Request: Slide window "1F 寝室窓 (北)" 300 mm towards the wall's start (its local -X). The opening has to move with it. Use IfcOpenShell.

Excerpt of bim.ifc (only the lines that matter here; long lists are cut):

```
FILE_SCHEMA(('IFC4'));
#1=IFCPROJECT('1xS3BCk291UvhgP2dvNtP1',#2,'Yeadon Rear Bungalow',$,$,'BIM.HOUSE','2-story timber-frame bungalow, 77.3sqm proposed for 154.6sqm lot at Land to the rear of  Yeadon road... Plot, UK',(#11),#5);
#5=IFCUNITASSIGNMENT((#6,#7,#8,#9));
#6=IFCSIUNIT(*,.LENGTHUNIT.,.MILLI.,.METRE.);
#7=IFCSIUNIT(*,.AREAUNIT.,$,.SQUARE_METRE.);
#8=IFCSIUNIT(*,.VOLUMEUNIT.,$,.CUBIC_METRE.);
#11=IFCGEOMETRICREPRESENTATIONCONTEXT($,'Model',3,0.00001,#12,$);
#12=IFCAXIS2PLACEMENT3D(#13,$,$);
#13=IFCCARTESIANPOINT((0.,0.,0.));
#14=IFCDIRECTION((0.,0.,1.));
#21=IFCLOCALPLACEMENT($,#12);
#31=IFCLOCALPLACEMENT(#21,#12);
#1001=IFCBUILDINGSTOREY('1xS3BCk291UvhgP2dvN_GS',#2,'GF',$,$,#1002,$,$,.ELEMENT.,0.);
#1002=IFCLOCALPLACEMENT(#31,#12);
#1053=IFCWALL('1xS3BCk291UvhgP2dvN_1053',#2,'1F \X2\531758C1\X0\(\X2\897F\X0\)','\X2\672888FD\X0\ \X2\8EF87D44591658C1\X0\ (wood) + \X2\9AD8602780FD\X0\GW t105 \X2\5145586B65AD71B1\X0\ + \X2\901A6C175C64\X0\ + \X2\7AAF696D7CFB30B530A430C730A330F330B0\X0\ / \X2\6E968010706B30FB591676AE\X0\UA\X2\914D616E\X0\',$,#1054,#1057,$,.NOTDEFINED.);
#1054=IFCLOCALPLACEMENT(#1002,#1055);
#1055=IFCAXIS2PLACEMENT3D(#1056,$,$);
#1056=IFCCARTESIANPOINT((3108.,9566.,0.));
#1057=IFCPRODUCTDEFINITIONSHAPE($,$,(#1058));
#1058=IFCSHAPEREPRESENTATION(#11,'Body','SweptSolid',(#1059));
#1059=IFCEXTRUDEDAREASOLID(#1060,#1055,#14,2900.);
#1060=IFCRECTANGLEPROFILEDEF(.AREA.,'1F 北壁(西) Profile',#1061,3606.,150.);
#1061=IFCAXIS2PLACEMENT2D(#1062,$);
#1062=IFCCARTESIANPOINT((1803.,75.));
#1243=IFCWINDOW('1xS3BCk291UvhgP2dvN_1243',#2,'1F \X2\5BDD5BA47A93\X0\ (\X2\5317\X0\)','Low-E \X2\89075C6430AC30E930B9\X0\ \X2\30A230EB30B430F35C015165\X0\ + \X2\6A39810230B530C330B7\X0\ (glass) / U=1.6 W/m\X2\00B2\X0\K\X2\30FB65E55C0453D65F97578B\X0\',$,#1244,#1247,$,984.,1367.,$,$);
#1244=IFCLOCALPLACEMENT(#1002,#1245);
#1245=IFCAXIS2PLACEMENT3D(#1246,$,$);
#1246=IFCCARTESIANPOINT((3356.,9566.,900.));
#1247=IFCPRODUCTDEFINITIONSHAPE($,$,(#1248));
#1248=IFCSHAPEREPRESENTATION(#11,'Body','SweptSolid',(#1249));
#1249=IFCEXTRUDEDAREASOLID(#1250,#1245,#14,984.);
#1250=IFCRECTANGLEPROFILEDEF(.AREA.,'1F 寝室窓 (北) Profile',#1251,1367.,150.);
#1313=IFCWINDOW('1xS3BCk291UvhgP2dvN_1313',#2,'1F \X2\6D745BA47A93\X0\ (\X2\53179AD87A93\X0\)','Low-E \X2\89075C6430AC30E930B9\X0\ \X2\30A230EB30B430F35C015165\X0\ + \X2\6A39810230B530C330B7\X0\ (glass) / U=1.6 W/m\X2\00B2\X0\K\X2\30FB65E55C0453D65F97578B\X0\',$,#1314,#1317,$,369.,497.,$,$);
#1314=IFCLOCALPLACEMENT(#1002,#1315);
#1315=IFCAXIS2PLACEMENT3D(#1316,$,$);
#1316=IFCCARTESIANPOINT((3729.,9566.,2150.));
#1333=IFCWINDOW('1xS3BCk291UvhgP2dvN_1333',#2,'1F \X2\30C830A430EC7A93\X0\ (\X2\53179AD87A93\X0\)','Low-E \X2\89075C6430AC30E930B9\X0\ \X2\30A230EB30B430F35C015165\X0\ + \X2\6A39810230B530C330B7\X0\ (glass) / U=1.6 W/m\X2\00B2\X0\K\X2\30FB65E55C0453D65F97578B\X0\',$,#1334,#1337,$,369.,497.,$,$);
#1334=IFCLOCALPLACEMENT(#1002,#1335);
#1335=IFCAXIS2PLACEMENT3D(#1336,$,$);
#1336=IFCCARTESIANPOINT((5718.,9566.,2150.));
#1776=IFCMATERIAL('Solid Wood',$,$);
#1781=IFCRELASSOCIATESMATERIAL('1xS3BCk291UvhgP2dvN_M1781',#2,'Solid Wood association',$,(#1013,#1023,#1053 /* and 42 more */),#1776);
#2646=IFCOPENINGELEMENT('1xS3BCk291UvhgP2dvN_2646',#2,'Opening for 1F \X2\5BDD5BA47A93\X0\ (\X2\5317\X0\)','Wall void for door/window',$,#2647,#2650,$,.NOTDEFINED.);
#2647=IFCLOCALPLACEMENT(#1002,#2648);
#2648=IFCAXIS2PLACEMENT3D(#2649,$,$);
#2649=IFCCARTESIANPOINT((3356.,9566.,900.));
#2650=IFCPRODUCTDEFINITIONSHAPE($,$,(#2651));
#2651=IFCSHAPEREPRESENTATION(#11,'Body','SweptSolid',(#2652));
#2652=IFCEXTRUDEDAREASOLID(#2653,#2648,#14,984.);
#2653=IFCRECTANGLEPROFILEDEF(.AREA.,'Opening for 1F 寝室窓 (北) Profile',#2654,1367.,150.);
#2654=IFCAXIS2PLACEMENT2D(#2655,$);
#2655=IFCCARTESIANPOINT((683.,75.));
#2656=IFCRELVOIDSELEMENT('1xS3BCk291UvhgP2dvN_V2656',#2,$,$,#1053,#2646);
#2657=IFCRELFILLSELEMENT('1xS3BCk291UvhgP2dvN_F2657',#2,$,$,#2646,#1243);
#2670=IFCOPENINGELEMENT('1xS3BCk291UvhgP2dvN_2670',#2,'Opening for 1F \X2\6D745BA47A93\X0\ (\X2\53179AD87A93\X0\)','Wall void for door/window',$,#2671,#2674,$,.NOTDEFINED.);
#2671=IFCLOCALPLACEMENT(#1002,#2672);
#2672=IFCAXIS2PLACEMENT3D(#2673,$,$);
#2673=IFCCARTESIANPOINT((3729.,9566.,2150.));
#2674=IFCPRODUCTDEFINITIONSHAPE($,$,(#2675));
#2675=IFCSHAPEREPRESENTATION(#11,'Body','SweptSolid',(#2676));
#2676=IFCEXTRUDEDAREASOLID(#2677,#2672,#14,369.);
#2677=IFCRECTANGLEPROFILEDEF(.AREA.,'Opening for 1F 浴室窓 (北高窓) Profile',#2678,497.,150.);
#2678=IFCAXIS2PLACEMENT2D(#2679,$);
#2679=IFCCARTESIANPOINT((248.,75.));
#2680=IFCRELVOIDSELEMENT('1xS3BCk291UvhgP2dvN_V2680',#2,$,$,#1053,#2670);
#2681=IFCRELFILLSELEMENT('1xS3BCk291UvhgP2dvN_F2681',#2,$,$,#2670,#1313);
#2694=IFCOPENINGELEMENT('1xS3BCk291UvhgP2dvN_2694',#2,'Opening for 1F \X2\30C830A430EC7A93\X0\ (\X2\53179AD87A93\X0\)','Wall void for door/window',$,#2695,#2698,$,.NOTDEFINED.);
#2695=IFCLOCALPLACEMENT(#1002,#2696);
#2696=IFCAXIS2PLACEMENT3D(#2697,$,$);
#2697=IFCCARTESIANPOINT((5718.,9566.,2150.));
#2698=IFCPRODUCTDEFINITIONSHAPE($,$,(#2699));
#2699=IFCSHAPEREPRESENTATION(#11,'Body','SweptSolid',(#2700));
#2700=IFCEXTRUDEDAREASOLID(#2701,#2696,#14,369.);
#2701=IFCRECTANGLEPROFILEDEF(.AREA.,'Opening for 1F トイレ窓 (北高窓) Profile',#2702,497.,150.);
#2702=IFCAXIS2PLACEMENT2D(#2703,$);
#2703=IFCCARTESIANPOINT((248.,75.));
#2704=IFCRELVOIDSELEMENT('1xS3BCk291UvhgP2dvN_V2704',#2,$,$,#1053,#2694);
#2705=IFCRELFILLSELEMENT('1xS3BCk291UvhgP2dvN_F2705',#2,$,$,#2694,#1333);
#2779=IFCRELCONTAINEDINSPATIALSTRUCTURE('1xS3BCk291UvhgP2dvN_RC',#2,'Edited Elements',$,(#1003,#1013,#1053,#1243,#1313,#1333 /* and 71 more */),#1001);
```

```python
import ifcopenshell
import ifcopenshell.api.geometry
import ifcopenshell.util.placement
import ifcopenshell.util.unit

model = ifcopenshell.open("bim.ifc")
unit_scale = ifcopenshell.util.unit.calculate_unit_scale(model)

window = model.by_guid("1xS3BCk291UvhgP2dvN_1243")
opening = window.FillsVoids[0].RelatingOpeningElement
wall = opening.VoidsElements[0].RelatingBuildingElement

wall_matrix = ifcopenshell.util.placement.get_local_placement(wall.ObjectPlacement)
shift = wall_matrix[:3, 0] * -0.3 / unit_scale
before = ifcopenshell.util.placement.get_local_placement(window.ObjectPlacement)[:3, 3].copy()

# The window is not placed relative to its opening, so move both.
for product in (opening, window):
    matrix = ifcopenshell.util.placement.get_local_placement(product.ObjectPlacement)
    matrix[:3, 3] += shift
    ifcopenshell.api.geometry.edit_object_placement(model, product=product, matrix=matrix, is_si=False)

after = ifcopenshell.util.placement.get_local_placement(window.ObjectPlacement)[:3, 3]
print("window moved by", (after - before).round(3) + 0.0)

model.write("bim-out.ifc")
```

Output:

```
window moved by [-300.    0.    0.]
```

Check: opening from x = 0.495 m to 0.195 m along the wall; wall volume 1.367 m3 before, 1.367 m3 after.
